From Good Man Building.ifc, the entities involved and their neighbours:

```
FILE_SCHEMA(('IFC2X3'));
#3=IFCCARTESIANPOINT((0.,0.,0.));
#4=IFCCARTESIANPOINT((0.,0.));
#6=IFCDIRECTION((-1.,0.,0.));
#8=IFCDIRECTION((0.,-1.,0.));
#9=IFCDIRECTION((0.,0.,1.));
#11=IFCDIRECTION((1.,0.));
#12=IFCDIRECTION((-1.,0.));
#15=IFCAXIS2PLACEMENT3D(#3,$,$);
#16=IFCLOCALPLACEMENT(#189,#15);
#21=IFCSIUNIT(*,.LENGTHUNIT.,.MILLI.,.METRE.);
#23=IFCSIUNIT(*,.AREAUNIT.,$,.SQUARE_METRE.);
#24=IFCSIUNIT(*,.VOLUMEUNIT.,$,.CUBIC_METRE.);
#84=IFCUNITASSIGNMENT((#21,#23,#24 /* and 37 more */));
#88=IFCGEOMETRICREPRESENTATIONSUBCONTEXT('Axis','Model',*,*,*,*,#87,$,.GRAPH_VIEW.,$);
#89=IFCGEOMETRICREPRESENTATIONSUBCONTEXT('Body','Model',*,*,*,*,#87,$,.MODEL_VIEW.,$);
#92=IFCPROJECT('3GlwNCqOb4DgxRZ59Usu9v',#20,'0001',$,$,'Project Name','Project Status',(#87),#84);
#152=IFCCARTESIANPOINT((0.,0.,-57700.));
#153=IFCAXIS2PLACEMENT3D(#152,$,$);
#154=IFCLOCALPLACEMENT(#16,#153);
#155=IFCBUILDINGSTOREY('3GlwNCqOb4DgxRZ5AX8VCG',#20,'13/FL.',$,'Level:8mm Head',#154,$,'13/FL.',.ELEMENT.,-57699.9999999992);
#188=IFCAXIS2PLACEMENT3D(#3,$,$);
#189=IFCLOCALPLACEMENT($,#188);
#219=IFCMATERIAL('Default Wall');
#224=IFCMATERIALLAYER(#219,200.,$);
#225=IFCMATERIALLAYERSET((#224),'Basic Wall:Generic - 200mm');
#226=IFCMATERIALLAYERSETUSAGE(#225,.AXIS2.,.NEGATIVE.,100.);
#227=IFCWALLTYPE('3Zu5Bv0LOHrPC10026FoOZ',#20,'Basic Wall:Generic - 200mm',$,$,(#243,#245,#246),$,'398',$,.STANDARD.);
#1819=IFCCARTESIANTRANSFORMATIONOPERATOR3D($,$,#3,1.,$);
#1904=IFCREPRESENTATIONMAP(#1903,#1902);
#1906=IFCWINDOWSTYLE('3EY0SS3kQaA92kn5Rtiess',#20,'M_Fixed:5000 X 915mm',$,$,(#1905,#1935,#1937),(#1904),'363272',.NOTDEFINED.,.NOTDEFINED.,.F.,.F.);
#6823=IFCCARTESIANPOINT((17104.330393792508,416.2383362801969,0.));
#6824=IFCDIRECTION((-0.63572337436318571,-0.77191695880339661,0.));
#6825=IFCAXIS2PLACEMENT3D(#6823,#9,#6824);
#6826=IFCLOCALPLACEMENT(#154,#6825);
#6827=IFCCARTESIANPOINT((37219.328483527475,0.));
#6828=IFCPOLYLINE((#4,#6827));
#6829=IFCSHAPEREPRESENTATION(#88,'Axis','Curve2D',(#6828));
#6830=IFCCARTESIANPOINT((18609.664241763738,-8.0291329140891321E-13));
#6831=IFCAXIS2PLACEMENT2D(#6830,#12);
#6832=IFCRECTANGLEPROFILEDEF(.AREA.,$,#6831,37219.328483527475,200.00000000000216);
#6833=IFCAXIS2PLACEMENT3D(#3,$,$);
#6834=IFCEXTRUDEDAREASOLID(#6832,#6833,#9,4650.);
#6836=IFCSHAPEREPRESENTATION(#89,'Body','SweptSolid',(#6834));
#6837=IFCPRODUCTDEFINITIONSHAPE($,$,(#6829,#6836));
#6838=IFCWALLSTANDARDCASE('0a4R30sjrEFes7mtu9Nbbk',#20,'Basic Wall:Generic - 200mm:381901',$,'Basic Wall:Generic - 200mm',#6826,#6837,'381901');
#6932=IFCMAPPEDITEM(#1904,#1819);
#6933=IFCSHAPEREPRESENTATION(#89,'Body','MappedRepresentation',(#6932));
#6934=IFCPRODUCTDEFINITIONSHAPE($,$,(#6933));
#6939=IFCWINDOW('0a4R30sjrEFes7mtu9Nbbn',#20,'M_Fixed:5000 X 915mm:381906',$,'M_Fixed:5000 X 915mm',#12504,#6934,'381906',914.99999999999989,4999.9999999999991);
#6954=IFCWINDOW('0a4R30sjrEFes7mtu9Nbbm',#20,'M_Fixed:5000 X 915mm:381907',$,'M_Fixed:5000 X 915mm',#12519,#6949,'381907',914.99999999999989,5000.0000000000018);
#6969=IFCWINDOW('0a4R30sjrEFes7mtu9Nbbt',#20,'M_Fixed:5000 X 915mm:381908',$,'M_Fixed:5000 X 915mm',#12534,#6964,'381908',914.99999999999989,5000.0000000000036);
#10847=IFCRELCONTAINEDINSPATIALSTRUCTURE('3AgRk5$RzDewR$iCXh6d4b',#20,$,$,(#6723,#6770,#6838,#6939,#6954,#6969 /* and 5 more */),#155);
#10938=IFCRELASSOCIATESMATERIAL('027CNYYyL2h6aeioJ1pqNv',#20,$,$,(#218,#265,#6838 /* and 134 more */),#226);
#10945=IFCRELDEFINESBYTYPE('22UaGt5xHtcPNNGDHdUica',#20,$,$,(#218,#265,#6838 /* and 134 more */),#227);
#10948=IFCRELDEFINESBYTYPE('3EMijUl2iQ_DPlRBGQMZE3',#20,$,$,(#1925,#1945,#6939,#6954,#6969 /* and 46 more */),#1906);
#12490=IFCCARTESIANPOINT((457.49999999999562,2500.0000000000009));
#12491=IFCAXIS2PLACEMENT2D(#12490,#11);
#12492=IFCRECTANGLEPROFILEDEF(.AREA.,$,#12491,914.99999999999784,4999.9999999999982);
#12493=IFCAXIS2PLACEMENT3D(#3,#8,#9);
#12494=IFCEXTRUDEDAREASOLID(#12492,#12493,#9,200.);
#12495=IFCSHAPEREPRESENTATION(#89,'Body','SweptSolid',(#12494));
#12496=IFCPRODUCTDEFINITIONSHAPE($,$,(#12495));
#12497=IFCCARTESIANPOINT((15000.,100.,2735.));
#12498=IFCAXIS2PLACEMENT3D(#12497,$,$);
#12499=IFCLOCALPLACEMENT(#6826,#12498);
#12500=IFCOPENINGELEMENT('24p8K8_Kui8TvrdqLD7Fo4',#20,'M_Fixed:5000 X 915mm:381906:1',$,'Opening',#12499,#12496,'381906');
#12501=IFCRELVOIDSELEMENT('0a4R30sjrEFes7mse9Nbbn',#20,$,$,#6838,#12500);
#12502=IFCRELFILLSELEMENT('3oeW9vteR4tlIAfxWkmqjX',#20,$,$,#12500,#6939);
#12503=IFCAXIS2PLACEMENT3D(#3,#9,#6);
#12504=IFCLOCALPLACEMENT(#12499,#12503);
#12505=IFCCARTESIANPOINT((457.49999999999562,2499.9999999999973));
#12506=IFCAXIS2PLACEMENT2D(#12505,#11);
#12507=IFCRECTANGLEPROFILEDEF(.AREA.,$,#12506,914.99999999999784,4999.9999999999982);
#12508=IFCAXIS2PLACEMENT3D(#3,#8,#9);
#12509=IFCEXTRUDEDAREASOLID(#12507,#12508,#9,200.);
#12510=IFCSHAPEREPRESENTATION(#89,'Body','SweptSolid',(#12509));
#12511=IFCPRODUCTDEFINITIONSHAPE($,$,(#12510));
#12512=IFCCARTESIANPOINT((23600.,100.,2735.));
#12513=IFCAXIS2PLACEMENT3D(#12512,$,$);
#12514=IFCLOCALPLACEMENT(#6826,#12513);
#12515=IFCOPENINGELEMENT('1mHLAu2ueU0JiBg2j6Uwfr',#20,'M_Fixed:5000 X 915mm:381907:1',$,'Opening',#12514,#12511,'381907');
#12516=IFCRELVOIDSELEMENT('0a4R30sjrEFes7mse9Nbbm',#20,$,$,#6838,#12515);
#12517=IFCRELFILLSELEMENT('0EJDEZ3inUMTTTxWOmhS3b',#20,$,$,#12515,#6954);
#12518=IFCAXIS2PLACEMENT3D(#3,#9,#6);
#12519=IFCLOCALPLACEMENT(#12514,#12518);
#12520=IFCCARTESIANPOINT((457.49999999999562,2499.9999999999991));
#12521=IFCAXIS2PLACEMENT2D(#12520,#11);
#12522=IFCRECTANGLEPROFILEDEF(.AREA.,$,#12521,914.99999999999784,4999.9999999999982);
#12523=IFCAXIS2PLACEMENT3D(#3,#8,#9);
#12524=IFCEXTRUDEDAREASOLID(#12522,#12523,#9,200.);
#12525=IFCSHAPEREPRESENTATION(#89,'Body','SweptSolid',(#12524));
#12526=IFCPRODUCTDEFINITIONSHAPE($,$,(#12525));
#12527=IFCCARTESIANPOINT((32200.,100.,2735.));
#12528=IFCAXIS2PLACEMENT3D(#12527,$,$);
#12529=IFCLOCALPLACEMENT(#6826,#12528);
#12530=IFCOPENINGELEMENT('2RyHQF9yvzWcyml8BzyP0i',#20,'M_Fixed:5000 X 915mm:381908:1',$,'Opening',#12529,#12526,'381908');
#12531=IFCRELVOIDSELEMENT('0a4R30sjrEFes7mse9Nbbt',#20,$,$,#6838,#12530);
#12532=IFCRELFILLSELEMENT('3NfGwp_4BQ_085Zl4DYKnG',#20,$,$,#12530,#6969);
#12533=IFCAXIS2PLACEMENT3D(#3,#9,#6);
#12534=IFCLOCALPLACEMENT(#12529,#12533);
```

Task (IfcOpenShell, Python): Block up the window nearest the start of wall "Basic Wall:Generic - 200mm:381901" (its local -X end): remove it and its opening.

```python
import ifcopenshell
import ifcopenshell.api.feature
import ifcopenshell.api.root
import ifcopenshell.geom
import ifcopenshell.util.shape

model = ifcopenshell.open("Good Man Building.ifc")
settings = ifcopenshell.geom.settings()


def volume(element):
    """Net volume in cubic metres, openings subtracted."""
    shape = ifcopenshell.geom.create_shape(settings, element)
    return ifcopenshell.util.shape.get_volume(shape.geometry)


window = model.by_guid("0a4R30sjrEFes7mtu9Nbbn")
opening = window.FillsVoids[0].RelatingOpeningElement
wall = opening.VoidsElements[0].RelatingBuildingElement
before = volume(wall)

ifcopenshell.api.root.remove_product(model, product=window)
ifcopenshell.api.feature.remove_feature(model, feature=opening)

after = volume(wall)

print(f"wall volume {before:.3f} -> {after:.3f} m3")

model.write("Good Man Building-out.ifc")
```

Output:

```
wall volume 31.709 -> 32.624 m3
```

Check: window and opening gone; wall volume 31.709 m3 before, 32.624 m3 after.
